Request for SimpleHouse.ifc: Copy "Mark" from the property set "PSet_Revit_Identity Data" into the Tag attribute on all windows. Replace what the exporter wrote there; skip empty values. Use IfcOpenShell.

First a look at what the model holds.

```python
import ifcopenshell
import ifcopenshell.util.element

model = ifcopenshell.open("SimpleHouse.ifc")
print(model.schema)
windows = model.by_type("IfcWindow")
print(len(windows), "windows")
for e in windows[:8]:
    source = ifcopenshell.util.element.get_pset(e, "PSet_Revit_Identity Data", "Mark")
    target = e.Tag
    print(e.id(), repr(source), repr(target), sep=" | ")
```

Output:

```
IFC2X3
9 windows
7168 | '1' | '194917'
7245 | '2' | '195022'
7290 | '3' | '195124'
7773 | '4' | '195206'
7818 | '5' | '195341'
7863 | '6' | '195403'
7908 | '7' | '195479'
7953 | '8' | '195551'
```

```python
import ifcopenshell
import ifcopenshell.util.element

model = ifcopenshell.open("SimpleHouse.ifc")

count = 0
for e in model.by_type("IfcWindow"):
    value = ifcopenshell.util.element.get_pset(e, "PSet_Revit_Identity Data", "Mark")
    current = e.Tag
    if not value or not value.strip() or current == value:
        continue
    e.Tag = value
    count += 1

print(count, "windows updated")

model.write("SimpleHouse_rev.ifc")
```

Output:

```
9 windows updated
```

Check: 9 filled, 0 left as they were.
